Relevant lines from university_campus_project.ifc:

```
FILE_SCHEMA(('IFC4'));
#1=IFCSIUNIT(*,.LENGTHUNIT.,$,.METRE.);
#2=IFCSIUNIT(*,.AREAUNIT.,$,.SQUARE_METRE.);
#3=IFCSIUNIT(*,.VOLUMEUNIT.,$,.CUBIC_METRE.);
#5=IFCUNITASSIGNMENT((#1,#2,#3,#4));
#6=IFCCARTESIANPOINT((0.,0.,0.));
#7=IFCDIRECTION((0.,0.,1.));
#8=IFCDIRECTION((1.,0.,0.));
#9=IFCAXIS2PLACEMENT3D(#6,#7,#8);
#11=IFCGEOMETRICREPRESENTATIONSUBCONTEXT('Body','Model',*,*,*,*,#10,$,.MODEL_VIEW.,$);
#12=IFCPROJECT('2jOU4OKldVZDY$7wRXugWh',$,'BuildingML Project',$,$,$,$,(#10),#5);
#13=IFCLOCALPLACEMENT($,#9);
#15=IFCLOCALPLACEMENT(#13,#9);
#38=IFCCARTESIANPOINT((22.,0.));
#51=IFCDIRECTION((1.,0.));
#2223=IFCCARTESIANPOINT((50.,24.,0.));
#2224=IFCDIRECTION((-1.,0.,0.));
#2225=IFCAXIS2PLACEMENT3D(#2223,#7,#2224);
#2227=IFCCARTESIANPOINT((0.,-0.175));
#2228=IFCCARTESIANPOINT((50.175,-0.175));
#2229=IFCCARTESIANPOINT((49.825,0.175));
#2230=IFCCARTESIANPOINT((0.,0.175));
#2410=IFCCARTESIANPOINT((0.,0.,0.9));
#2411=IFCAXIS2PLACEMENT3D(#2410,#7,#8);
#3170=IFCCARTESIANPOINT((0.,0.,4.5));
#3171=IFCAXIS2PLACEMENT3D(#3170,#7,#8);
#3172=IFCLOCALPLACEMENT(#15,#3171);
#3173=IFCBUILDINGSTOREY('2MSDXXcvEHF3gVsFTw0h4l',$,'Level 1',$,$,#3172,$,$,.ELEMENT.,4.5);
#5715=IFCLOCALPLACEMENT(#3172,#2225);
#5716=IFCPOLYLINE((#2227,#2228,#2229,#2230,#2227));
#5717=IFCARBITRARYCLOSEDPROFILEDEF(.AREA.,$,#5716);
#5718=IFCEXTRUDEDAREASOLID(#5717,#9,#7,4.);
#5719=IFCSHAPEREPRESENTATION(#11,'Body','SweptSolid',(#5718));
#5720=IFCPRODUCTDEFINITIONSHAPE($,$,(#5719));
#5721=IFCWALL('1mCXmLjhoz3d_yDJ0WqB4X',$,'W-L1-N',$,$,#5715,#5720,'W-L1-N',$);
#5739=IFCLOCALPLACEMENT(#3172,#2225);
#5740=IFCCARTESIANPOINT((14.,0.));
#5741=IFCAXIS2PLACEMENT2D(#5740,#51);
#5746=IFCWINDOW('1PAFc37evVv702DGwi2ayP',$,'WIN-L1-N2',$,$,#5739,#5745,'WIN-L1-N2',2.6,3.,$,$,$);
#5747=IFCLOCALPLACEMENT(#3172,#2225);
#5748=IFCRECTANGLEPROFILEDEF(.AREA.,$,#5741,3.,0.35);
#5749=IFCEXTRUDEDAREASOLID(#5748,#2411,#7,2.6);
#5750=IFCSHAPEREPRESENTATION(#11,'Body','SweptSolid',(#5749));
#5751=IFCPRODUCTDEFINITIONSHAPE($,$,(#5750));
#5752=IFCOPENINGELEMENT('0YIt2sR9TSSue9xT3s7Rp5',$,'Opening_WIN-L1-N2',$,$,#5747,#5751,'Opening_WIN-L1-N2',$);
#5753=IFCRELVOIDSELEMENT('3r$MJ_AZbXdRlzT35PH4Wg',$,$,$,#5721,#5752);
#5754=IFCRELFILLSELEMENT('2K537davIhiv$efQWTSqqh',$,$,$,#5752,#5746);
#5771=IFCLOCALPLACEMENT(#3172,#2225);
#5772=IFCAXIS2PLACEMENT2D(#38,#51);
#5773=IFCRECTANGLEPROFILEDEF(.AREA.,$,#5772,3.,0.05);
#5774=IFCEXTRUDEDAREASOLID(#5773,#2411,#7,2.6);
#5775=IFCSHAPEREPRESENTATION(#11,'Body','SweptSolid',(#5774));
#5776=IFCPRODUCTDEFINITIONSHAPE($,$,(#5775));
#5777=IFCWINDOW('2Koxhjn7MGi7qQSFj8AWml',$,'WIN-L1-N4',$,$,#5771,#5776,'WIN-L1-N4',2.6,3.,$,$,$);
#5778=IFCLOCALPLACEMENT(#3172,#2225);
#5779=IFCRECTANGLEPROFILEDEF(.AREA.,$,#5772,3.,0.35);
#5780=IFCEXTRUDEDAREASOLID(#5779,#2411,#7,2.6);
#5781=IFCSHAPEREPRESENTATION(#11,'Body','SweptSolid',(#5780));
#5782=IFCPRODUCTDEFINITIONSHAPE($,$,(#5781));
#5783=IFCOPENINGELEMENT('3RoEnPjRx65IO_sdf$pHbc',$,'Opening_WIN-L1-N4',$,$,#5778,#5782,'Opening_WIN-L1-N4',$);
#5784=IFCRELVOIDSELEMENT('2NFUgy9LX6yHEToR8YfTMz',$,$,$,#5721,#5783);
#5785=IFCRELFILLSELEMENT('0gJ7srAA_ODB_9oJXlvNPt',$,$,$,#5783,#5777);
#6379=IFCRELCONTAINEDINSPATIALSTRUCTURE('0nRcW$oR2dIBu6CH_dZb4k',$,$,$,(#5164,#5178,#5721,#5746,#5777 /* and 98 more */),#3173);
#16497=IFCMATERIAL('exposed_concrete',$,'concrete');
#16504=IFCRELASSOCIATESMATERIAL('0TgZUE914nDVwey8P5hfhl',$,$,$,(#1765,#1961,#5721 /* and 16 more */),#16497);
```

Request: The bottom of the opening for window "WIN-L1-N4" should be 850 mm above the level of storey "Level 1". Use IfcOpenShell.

```python
import numpy as np
import ifcopenshell
import ifcopenshell.api.geometry
import ifcopenshell.geom
import ifcopenshell.util.element
import ifcopenshell.util.placement
import ifcopenshell.util.shape
import ifcopenshell.util.unit

model = ifcopenshell.open("university_campus_project.ifc")
unit_scale = ifcopenshell.util.unit.calculate_unit_scale(model)

window = model.by_guid("2Koxhjn7MGi7qQSFj8AWml")
opening = window.FillsVoids[0].RelatingOpeningElement
storey = ifcopenshell.util.element.get_container(window, ifc_class="IfcBuildingStorey")
level = ifcopenshell.util.placement.get_local_placement(storey.ObjectPlacement)[2, 3]

# The opening's origin need not be at the sill, so measure its lowest point.
shape = ifcopenshell.geom.create_shape(ifcopenshell.geom.settings(), opening)
bottom = ifcopenshell.util.shape.get_shape_bottom_elevation(shape, shape.geometry) / unit_scale
dz = level + 0.85 / unit_scale - bottom

shift = np.array([0.0, 0.0, dz])
# The window is not placed relative to its opening, so move both.
for product in (opening, window):
    matrix = ifcopenshell.util.placement.get_local_placement(product.ObjectPlacement)
    matrix[:3, 3] += shift
    ifcopenshell.api.geometry.edit_object_placement(model, product=product, matrix=matrix, is_si=False)

print(f"moved by {dz * unit_scale:+.3f} m")

model.write("university_campus_project_edited.ifc")
```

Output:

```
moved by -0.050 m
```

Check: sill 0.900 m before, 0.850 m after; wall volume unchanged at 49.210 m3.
